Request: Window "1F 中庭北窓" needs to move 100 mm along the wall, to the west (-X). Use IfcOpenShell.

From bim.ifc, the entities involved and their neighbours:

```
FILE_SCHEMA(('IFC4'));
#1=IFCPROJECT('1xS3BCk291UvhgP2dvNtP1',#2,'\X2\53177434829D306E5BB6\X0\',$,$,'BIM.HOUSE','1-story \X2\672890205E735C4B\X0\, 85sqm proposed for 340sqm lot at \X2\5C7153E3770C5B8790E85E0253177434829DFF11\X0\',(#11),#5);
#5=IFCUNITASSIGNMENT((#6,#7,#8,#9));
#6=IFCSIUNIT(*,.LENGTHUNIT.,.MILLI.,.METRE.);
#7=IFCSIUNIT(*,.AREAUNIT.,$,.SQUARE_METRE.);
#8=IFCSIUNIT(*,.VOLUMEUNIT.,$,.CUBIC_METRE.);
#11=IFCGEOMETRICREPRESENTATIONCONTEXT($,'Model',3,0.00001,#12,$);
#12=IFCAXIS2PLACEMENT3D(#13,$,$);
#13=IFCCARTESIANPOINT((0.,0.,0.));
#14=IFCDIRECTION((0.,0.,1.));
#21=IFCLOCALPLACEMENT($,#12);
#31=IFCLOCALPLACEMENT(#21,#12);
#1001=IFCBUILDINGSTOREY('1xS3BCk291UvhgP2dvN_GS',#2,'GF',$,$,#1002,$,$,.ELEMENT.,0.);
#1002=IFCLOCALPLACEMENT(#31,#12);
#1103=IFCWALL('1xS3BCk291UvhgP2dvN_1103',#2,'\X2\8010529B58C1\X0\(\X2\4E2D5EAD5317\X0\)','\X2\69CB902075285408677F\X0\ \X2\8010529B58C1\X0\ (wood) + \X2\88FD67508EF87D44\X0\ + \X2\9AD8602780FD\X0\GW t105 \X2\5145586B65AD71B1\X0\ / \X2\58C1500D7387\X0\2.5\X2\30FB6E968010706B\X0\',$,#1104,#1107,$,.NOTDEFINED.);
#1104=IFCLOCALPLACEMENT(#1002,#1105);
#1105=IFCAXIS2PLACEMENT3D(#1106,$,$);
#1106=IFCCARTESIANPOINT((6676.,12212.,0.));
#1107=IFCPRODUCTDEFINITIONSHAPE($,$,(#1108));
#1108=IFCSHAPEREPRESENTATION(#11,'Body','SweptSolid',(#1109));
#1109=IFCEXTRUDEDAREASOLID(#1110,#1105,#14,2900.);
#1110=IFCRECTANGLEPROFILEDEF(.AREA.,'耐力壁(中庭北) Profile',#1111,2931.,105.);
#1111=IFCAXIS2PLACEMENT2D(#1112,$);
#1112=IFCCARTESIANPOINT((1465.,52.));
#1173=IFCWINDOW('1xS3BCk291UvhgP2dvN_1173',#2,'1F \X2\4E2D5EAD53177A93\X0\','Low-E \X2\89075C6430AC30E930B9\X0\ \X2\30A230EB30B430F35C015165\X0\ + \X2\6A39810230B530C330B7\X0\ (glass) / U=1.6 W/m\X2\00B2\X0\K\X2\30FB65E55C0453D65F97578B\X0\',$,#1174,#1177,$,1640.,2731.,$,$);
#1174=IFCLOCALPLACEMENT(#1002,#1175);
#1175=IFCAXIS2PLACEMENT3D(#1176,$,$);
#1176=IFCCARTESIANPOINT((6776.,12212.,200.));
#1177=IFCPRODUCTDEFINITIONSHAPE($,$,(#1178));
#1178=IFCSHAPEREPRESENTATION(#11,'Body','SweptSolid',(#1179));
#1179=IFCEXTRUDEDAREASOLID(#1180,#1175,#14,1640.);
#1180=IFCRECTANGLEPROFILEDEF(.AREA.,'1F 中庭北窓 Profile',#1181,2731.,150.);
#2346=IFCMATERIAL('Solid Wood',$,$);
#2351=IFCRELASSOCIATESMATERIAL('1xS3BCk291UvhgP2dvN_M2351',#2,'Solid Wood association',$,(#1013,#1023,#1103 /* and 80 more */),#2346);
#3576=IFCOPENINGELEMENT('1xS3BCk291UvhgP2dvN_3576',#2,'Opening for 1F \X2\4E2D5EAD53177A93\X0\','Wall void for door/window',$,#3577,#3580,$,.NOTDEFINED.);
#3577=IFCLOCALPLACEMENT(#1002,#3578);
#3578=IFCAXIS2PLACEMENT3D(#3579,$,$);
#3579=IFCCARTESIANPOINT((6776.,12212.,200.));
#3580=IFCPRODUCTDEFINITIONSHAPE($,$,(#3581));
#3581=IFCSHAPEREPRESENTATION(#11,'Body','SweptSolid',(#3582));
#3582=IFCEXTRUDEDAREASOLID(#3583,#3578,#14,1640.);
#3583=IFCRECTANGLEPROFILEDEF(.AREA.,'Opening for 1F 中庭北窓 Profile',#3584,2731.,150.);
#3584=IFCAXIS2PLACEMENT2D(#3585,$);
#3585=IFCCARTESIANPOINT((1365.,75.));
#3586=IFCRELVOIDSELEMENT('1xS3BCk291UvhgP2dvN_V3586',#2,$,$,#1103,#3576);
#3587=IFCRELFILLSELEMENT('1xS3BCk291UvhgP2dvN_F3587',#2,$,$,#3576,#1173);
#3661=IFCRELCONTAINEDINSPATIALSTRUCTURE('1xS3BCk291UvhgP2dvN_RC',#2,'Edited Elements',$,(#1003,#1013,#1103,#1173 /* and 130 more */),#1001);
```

```python
import ifcopenshell
import ifcopenshell.api.geometry
import ifcopenshell.util.placement
import ifcopenshell.util.unit

model = ifcopenshell.open("bim.ifc")
unit_scale = ifcopenshell.util.unit.calculate_unit_scale(model)

window = model.by_guid("1xS3BCk291UvhgP2dvN_1173")
opening = window.FillsVoids[0].RelatingOpeningElement
wall = opening.VoidsElements[0].RelatingBuildingElement

wall_matrix = ifcopenshell.util.placement.get_local_placement(wall.ObjectPlacement)
shift = wall_matrix[:3, 0] * -0.1 / unit_scale
before = ifcopenshell.util.placement.get_local_placement(window.ObjectPlacement)[:3, 3].copy()

# The window is not placed relative to its opening, so move both.
for product in (opening, window):
    matrix = ifcopenshell.util.placement.get_local_placement(product.ObjectPlacement)
    matrix[:3, 3] += shift
    ifcopenshell.api.geometry.edit_object_placement(model, product=product, matrix=matrix, is_si=False)

after = ifcopenshell.util.placement.get_local_placement(window.ObjectPlacement)[:3, 3]
print("window moved by", (after - before).round(3) + 0.0)

model.write("bim_edited.ifc")
```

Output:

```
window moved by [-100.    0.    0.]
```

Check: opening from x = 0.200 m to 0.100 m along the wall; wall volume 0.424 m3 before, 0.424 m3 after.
